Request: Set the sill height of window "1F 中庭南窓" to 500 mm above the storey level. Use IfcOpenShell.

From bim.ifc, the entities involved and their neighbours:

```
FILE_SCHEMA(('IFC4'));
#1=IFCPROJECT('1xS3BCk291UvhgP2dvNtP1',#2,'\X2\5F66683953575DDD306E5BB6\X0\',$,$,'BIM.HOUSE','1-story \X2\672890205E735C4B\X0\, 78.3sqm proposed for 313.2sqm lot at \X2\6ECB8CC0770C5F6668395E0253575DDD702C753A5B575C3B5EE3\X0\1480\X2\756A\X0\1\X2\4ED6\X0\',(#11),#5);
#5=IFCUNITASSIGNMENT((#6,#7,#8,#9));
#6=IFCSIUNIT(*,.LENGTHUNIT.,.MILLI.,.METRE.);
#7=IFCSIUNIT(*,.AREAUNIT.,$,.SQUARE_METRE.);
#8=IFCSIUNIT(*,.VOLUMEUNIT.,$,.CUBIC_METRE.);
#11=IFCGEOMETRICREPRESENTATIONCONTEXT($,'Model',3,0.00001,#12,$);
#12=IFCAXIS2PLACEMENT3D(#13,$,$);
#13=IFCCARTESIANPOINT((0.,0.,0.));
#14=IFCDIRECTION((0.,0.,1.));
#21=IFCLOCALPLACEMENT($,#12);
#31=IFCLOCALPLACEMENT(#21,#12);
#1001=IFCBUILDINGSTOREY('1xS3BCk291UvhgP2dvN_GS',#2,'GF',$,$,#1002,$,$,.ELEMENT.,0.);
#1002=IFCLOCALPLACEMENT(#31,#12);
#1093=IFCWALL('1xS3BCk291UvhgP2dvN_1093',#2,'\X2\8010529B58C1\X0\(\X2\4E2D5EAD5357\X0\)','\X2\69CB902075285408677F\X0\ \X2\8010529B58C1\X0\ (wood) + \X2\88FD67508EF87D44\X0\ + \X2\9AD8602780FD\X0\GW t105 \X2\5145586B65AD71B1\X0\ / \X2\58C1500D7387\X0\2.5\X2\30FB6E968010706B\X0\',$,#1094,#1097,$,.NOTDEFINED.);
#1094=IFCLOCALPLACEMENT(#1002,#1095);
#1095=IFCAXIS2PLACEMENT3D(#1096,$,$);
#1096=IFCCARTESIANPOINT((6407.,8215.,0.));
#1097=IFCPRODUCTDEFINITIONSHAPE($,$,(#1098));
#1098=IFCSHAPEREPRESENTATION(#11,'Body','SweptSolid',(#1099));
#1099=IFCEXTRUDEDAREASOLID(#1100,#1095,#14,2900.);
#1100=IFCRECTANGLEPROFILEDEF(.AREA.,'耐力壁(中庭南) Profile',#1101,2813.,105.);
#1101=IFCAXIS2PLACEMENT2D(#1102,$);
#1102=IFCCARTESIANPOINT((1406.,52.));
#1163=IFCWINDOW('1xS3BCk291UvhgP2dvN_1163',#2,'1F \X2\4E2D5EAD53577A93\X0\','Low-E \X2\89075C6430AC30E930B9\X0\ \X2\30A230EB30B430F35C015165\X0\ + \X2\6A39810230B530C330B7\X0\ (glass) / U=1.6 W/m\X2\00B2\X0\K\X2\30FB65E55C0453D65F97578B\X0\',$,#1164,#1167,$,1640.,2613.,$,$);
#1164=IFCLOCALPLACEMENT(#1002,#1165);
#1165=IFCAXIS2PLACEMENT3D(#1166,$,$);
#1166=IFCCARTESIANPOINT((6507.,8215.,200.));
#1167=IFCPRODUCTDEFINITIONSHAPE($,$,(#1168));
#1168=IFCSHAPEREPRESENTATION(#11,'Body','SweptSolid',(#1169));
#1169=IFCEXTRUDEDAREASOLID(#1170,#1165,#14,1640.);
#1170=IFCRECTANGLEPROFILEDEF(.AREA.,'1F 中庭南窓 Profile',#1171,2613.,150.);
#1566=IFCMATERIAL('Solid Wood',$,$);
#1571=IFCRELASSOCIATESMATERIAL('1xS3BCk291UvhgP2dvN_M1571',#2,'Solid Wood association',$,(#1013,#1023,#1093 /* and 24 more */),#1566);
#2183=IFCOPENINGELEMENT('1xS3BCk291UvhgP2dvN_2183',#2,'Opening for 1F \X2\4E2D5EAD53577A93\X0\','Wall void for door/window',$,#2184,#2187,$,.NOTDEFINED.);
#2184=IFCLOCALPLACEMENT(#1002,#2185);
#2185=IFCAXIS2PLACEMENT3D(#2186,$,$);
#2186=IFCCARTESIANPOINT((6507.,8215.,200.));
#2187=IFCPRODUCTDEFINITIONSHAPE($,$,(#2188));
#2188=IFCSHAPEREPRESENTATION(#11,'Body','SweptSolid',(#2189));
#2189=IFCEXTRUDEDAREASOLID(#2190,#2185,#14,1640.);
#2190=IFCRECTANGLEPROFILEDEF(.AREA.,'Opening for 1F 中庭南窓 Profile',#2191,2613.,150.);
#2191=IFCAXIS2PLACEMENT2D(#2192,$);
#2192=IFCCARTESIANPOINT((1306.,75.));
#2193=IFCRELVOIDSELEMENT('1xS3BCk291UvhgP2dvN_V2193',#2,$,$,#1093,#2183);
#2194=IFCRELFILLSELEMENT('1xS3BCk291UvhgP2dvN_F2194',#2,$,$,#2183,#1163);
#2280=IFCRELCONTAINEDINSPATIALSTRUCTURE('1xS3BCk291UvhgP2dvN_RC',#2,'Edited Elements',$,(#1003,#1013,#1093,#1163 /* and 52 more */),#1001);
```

```python
import numpy as np
import ifcopenshell
import ifcopenshell.api.geometry
import ifcopenshell.geom
import ifcopenshell.util.element
import ifcopenshell.util.placement
import ifcopenshell.util.shape
import ifcopenshell.util.unit

model = ifcopenshell.open("bim.ifc")
unit_scale = ifcopenshell.util.unit.calculate_unit_scale(model)

window = model.by_id(1163)
opening = window.FillsVoids[0].RelatingOpeningElement
storey = ifcopenshell.util.element.get_container(window, ifc_class="IfcBuildingStorey")
level = ifcopenshell.util.placement.get_local_placement(storey.ObjectPlacement)[2, 3]

# The opening's origin need not be at the sill, so measure its lowest point.
shape = ifcopenshell.geom.create_shape(ifcopenshell.geom.settings(), opening)
bottom = ifcopenshell.util.shape.get_shape_bottom_elevation(shape, shape.geometry) / unit_scale
dz = level + 0.5 / unit_scale - bottom

shift = np.array([0.0, 0.0, dz])
# The window is not placed relative to its opening, so move both.
for product in (opening, window):
    matrix = ifcopenshell.util.placement.get_local_placement(product.ObjectPlacement)
    matrix[:3, 3] += shift
    ifcopenshell.api.geometry.edit_object_placement(model, product=product, matrix=matrix, is_si=False)

print(f"moved by {dz * unit_scale:+.3f} m")

model.write("bim_rev.ifc")
```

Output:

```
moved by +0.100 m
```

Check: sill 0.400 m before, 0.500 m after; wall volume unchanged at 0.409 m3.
